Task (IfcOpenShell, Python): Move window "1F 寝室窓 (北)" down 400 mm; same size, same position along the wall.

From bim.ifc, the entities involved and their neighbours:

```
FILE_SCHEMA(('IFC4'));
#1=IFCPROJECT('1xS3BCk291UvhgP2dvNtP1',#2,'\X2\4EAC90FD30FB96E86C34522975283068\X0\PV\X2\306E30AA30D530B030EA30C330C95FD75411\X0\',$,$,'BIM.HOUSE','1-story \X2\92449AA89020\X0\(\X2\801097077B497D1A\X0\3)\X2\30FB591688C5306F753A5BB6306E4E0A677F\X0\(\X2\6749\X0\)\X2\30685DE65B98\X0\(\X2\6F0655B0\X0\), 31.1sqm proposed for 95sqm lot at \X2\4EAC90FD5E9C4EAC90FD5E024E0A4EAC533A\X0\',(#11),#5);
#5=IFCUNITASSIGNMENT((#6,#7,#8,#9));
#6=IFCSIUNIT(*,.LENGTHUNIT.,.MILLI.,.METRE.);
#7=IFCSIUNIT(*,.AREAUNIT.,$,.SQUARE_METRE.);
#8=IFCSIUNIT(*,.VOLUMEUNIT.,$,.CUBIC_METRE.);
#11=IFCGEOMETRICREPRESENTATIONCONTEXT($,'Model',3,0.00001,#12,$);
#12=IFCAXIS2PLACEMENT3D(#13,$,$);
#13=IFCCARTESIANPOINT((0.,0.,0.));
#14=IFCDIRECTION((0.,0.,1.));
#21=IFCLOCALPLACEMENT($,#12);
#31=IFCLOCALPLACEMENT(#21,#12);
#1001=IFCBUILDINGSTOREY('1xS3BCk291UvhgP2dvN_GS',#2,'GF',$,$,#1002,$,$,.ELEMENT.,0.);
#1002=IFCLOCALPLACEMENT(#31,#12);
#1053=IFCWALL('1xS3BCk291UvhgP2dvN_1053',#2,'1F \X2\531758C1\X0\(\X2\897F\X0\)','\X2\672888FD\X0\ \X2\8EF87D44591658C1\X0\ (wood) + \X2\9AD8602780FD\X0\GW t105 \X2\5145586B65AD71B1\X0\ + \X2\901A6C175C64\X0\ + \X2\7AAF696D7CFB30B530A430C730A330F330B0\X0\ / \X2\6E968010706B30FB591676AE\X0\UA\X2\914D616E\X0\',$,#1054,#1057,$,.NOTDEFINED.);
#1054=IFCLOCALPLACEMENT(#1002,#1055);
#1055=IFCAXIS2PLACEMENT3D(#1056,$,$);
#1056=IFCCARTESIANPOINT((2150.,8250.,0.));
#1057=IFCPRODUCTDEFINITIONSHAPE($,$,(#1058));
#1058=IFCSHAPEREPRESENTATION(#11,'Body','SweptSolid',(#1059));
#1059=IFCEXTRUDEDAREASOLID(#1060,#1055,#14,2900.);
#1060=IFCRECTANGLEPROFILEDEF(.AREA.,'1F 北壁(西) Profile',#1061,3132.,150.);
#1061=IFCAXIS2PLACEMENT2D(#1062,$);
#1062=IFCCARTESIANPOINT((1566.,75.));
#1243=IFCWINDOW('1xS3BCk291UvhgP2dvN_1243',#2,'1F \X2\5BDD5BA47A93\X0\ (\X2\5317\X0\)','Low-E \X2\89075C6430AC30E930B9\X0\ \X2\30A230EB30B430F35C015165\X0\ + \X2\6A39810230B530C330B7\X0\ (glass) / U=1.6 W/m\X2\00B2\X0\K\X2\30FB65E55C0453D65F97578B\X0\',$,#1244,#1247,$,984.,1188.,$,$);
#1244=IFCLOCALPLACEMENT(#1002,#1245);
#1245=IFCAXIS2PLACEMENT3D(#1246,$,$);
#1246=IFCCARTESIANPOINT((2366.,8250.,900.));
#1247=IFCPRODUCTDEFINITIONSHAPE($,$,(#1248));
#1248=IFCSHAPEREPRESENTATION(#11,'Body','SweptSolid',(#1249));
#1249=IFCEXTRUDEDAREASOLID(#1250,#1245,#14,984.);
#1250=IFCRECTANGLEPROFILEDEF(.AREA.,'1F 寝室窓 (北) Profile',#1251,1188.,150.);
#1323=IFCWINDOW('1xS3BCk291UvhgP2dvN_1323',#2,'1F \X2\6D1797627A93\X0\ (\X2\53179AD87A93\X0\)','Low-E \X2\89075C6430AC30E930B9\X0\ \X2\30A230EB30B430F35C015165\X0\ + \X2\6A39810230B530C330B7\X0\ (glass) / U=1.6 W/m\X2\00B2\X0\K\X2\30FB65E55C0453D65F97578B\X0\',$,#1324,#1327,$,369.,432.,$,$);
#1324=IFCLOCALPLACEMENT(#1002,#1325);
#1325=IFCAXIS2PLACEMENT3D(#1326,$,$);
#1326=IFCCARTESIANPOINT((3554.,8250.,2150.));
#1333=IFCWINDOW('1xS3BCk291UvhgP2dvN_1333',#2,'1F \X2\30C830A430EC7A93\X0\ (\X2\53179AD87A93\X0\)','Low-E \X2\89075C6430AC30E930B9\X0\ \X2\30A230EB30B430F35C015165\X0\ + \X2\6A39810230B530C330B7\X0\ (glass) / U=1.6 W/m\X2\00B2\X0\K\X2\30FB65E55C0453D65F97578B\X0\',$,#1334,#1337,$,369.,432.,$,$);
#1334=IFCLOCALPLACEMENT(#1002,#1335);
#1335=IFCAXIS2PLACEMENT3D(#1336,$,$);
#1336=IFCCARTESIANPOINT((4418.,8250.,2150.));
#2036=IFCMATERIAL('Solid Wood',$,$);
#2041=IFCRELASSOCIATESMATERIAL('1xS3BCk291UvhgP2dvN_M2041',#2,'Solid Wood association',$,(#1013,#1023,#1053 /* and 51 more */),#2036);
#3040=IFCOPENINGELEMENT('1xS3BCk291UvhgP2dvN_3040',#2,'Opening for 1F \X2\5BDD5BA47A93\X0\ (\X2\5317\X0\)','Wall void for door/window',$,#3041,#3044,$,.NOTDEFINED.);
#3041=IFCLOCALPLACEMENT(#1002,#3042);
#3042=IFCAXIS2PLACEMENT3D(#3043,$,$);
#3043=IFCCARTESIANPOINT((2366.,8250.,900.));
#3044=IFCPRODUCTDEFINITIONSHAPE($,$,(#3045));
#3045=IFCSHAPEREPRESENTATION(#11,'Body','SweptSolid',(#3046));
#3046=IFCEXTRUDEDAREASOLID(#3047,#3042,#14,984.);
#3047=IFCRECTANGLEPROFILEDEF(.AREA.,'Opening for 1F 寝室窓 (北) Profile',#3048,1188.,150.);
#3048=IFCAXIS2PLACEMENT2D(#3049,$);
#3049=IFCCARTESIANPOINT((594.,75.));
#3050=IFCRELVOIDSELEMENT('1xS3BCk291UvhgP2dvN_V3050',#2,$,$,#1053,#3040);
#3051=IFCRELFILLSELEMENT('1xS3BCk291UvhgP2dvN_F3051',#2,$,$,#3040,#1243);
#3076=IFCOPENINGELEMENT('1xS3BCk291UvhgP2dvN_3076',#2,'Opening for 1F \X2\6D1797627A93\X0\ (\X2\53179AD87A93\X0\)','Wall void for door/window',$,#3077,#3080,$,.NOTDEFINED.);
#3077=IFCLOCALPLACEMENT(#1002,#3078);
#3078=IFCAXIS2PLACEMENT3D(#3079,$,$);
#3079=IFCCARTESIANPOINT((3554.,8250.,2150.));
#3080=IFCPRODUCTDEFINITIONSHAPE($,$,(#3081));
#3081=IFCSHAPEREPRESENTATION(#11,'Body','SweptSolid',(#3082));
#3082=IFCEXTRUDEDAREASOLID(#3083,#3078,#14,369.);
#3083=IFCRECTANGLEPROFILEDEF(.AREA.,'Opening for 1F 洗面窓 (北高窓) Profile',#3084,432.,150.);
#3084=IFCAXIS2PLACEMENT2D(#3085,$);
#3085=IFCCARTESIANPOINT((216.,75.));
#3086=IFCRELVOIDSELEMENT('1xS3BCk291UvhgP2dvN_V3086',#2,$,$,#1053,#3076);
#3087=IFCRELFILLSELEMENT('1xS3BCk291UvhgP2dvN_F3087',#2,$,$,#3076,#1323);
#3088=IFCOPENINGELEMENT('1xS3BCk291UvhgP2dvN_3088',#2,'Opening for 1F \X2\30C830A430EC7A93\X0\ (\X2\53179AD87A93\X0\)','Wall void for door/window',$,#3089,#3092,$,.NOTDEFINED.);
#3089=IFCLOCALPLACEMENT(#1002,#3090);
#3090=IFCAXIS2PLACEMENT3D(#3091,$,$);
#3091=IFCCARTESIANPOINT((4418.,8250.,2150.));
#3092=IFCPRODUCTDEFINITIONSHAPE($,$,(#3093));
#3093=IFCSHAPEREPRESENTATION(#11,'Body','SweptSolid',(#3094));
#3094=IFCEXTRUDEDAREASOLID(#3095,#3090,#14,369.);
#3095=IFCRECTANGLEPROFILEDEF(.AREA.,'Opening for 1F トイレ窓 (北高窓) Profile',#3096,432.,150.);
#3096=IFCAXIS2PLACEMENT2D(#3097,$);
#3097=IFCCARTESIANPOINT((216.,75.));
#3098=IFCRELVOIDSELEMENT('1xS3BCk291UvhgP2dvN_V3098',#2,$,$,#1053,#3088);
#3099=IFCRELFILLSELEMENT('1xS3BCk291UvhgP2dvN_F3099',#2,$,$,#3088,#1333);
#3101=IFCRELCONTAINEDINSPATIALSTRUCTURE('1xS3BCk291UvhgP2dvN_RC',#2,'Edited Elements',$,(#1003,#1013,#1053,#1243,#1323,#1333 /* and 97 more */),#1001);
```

```python
import numpy as np
import ifcopenshell
import ifcopenshell.api.geometry
import ifcopenshell.util.placement
import ifcopenshell.util.unit

model = ifcopenshell.open("bim.ifc")
unit_scale = ifcopenshell.util.unit.calculate_unit_scale(model)

window = model.by_guid("1xS3BCk291UvhgP2dvN_1243")
opening = window.FillsVoids[0].RelatingOpeningElement
dz = -0.4 / unit_scale

shift = np.array([0.0, 0.0, dz])
# The window is not placed relative to its opening, so move both.
for product in (opening, window):
    matrix = ifcopenshell.util.placement.get_local_placement(product.ObjectPlacement)
    matrix[:3, 3] += shift
    ifcopenshell.api.geometry.edit_object_placement(model, product=product, matrix=matrix, is_si=False)

print(f"moved by {dz * unit_scale:+.3f} m")

model.write("bim-out.ifc")
```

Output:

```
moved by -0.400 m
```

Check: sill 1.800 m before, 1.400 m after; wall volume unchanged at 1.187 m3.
